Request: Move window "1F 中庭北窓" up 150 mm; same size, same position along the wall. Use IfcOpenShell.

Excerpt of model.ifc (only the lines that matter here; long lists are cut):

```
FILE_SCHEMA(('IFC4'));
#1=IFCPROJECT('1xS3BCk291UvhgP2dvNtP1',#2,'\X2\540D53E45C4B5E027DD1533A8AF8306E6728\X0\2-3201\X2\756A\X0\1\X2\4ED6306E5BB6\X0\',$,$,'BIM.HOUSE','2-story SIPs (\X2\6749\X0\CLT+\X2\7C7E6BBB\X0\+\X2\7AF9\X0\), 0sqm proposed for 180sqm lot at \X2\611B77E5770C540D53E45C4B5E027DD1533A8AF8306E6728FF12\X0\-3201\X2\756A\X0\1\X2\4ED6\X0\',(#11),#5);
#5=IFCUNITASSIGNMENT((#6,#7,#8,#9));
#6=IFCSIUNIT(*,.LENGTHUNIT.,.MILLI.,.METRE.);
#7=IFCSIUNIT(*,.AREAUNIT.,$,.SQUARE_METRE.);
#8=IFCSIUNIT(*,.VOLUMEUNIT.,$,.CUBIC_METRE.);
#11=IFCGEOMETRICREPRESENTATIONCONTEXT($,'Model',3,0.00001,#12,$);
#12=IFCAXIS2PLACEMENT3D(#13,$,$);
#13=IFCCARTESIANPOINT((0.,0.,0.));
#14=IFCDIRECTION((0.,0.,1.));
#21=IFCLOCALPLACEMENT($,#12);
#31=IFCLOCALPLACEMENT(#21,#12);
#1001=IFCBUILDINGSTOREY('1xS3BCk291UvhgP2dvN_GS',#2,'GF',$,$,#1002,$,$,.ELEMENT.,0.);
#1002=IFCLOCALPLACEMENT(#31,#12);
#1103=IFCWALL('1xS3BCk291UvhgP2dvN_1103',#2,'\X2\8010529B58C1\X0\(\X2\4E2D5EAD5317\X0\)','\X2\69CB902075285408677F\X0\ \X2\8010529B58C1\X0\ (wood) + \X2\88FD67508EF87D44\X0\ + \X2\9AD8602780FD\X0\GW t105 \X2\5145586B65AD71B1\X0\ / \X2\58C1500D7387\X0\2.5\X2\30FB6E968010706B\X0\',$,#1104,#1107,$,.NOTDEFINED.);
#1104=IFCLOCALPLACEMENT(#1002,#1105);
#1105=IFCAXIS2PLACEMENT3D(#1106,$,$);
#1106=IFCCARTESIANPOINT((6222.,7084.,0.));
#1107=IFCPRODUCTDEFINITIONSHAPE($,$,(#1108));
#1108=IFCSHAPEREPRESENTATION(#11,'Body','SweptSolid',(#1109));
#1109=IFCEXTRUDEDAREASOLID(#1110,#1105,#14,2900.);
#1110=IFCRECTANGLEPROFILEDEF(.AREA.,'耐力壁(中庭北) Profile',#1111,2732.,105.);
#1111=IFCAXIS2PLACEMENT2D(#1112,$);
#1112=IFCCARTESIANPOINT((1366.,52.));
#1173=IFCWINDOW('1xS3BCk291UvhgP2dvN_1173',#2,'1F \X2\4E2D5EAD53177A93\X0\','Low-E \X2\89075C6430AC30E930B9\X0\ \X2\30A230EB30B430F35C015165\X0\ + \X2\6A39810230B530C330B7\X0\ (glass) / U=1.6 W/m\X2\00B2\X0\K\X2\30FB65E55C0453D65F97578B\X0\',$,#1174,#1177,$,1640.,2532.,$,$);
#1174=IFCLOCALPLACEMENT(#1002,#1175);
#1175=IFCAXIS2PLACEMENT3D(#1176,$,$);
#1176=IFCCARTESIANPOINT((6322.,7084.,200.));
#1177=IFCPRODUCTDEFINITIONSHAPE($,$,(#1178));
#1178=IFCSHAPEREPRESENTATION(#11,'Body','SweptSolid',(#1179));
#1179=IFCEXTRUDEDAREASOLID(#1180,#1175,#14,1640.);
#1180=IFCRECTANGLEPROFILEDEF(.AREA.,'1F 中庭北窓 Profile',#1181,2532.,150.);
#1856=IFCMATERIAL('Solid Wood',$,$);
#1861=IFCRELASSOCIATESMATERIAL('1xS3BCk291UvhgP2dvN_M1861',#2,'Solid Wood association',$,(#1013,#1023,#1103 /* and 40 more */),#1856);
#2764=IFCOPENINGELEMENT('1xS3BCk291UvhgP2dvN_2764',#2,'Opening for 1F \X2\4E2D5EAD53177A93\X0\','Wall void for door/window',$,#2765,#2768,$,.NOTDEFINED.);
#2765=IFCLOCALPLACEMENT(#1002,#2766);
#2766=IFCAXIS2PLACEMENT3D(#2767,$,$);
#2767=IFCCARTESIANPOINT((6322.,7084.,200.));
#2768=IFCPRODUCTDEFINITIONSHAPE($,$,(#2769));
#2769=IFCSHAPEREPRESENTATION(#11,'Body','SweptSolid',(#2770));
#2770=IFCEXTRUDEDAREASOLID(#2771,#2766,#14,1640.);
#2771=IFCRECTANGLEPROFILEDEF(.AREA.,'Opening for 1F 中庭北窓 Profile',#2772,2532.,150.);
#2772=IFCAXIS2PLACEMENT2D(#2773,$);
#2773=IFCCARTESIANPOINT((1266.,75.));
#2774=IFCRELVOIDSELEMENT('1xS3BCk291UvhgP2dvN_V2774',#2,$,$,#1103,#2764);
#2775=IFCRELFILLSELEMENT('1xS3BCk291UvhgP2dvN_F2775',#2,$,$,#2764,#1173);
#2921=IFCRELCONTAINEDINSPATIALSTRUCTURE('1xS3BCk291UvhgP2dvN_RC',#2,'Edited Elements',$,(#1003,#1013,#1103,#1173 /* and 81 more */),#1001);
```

```python
import numpy as np
import ifcopenshell
import ifcopenshell.api.geometry
import ifcopenshell.util.placement
import ifcopenshell.util.unit

model = ifcopenshell.open("model.ifc")
unit_scale = ifcopenshell.util.unit.calculate_unit_scale(model)

window = model.by_guid("1xS3BCk291UvhgP2dvN_1173")
opening = window.FillsVoids[0].RelatingOpeningElement
dz = 0.15 / unit_scale

shift = np.array([0.0, 0.0, dz])
# The window is not placed relative to its opening, so move both.
for product in (opening, window):
    matrix = ifcopenshell.util.placement.get_local_placement(product.ObjectPlacement)
    matrix[:3, 3] += shift
    ifcopenshell.api.geometry.edit_object_placement(model, product=product, matrix=matrix, is_si=False)

print(f"moved by {dz * unit_scale:+.3f} m")

model.write("model_v2.ifc")
```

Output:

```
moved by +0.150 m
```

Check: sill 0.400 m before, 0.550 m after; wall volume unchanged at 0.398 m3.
